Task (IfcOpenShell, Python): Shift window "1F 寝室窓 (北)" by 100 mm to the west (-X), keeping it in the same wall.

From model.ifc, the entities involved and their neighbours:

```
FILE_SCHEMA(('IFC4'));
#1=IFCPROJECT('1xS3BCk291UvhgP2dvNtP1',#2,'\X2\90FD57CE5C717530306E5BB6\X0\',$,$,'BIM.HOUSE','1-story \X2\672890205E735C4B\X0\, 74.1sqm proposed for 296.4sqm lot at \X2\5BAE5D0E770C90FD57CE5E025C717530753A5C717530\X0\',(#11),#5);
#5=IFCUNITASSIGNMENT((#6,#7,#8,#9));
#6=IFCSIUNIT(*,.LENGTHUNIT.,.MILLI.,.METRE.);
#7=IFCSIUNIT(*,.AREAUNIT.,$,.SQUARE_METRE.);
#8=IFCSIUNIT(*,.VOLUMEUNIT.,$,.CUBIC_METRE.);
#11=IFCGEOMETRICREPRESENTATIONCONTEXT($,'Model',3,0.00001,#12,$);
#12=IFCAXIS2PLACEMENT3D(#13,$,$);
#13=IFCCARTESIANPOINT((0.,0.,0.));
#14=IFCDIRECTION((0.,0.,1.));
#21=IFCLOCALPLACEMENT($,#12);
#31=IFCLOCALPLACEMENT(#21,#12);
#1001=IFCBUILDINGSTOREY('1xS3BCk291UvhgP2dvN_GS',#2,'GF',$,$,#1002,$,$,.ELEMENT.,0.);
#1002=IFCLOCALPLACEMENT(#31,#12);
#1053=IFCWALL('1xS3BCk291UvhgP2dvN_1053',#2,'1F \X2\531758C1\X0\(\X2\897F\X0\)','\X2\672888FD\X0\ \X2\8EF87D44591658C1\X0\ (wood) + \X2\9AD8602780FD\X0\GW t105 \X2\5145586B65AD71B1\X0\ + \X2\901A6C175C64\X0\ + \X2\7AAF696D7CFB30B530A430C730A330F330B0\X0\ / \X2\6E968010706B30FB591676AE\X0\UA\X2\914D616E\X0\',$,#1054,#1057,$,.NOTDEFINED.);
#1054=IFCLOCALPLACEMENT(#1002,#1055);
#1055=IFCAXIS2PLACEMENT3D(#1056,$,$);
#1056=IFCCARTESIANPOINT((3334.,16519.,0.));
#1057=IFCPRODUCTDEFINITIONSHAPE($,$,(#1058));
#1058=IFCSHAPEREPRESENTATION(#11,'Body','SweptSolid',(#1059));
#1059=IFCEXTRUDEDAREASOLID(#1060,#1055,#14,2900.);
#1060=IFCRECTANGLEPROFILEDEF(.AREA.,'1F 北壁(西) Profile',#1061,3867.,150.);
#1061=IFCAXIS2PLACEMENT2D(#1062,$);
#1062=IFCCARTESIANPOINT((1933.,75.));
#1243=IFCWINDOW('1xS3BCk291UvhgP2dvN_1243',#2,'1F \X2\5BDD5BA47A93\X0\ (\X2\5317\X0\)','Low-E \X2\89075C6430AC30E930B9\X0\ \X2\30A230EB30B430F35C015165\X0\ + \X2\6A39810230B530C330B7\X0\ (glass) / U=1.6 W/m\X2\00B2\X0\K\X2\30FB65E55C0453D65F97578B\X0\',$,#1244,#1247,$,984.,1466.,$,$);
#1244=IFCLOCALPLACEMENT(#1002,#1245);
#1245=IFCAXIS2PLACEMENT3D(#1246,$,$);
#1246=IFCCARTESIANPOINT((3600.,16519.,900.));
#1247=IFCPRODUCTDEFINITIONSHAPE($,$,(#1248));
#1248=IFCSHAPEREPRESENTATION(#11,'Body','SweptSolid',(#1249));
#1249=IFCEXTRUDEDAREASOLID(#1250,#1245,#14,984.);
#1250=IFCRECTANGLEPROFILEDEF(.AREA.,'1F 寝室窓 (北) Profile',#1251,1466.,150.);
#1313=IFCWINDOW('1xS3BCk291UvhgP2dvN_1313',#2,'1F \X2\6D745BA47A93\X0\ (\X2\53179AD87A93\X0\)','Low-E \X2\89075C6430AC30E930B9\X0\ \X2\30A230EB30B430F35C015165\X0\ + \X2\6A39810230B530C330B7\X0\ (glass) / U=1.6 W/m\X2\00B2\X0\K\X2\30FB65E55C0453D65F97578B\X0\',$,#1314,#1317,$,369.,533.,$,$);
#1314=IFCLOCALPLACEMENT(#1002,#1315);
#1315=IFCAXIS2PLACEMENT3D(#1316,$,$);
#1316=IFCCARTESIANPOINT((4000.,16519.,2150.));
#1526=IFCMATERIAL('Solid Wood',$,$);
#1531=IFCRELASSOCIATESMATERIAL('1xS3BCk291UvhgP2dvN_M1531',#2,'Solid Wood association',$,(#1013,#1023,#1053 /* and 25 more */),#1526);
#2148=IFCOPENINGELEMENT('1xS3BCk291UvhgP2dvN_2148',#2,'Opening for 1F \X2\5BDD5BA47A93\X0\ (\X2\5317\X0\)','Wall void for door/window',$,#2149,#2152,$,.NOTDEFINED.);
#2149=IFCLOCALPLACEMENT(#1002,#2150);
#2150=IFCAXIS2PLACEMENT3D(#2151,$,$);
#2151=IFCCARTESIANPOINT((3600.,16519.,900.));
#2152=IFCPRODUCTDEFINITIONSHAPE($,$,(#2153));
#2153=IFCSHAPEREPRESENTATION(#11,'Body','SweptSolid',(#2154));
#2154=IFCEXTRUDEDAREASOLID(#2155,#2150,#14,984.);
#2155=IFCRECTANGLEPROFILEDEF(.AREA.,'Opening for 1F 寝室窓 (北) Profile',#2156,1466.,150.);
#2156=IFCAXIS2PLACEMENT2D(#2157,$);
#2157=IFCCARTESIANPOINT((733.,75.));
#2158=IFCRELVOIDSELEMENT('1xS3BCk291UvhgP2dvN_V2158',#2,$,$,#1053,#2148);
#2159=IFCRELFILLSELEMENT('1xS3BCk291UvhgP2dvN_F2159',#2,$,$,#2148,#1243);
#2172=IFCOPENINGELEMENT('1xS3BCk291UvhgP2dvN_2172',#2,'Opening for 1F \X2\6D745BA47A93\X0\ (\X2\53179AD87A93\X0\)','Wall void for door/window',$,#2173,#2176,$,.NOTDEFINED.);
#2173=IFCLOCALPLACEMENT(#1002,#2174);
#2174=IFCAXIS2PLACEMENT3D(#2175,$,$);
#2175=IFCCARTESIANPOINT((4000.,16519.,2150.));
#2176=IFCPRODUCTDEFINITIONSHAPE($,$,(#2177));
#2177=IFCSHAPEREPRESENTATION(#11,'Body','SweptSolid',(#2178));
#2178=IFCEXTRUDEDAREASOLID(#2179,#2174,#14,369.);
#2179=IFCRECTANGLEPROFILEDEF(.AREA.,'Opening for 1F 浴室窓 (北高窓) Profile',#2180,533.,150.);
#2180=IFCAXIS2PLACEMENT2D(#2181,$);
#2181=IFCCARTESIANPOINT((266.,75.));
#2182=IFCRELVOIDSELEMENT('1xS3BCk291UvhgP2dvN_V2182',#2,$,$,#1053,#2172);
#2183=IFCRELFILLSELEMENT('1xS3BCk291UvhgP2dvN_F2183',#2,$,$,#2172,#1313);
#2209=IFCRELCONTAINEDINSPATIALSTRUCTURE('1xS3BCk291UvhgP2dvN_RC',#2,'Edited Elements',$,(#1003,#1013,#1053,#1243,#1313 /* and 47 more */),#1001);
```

```python
import ifcopenshell
import ifcopenshell.api.geometry
import ifcopenshell.util.placement
import ifcopenshell.util.unit

model = ifcopenshell.open("model.ifc")
unit_scale = ifcopenshell.util.unit.calculate_unit_scale(model)

window = model.by_guid("1xS3BCk291UvhgP2dvN_1243")
opening = window.FillsVoids[0].RelatingOpeningElement
wall = opening.VoidsElements[0].RelatingBuildingElement

wall_matrix = ifcopenshell.util.placement.get_local_placement(wall.ObjectPlacement)
shift = wall_matrix[:3, 0] * -0.1 / unit_scale
before = ifcopenshell.util.placement.get_local_placement(window.ObjectPlacement)[:3, 3].copy()

# The window is not placed relative to its opening, so move both.
for product in (opening, window):
    matrix = ifcopenshell.util.placement.get_local_placement(product.ObjectPlacement)
    matrix[:3, 3] += shift
    ifcopenshell.api.geometry.edit_object_placement(model, product=product, matrix=matrix, is_si=False)

after = ifcopenshell.util.placement.get_local_placement(window.ObjectPlacement)[:3, 3]
print("window moved by", (after - before).round(3) + 0.0)

model.write("model_edited.ifc")
```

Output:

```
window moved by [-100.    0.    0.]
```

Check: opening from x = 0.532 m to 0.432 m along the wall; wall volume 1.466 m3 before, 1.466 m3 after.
